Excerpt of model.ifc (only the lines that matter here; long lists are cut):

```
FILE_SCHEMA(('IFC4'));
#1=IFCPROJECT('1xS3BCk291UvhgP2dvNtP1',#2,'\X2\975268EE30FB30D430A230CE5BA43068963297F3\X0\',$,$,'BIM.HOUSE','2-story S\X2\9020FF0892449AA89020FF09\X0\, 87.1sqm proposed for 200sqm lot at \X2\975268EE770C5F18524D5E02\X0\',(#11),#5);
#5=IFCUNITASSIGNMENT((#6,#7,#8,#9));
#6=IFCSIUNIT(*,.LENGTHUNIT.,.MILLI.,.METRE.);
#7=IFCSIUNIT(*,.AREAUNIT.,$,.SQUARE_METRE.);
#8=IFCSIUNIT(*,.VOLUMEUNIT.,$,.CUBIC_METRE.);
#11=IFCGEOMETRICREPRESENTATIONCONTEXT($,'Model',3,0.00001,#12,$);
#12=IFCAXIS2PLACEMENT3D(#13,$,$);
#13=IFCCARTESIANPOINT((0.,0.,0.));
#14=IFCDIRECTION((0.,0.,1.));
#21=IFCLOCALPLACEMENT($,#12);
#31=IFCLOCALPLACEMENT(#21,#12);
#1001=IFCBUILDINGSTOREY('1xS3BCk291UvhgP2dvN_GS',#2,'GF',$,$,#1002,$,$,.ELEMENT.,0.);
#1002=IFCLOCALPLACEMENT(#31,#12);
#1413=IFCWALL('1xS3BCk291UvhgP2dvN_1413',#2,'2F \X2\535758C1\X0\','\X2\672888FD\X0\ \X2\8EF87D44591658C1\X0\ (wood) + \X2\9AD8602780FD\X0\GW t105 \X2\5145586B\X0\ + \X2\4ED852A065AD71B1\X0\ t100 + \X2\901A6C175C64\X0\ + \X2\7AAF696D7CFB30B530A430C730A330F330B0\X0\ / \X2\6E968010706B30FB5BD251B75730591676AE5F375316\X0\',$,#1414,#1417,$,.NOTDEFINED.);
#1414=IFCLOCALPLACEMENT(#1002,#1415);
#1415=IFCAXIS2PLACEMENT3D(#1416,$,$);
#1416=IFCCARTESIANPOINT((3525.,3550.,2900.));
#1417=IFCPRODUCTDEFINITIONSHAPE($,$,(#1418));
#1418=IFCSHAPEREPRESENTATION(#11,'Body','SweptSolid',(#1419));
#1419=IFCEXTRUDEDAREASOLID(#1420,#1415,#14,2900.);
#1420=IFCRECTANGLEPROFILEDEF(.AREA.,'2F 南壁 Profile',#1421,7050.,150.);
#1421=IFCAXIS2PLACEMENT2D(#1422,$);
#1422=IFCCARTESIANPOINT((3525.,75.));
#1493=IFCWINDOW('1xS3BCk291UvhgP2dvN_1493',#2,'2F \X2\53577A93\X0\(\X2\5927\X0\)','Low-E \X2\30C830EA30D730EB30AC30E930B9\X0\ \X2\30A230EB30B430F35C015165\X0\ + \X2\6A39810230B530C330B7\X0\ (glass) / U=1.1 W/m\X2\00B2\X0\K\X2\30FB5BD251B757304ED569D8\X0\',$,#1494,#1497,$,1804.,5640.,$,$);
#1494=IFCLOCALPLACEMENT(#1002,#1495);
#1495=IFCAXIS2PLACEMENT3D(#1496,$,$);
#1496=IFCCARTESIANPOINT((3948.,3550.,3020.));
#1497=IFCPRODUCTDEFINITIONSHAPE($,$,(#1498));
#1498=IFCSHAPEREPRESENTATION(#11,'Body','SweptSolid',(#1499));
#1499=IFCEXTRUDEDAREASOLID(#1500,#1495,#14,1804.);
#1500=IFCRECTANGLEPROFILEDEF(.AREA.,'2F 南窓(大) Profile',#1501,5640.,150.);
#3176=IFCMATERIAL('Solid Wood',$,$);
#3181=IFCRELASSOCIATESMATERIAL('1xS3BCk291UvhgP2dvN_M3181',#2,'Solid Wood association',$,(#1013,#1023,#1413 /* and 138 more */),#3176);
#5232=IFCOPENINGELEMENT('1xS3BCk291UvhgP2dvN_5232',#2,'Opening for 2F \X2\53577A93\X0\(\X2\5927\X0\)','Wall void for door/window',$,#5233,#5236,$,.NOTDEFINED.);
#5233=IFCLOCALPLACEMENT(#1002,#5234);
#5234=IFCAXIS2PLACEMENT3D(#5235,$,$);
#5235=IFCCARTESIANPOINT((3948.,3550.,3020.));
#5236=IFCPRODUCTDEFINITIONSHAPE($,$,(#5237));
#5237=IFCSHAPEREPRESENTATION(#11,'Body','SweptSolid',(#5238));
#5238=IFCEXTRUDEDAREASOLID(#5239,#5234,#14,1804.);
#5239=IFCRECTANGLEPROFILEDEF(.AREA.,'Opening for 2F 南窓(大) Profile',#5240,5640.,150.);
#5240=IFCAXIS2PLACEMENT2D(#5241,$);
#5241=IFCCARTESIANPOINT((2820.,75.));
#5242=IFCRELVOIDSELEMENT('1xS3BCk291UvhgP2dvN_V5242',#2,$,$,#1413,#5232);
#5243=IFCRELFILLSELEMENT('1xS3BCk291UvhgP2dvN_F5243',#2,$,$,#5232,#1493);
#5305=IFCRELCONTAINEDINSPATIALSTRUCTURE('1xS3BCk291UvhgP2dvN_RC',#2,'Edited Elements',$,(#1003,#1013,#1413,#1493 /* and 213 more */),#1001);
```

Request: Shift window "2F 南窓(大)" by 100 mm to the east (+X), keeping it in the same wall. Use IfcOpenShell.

```python
import ifcopenshell
import ifcopenshell.api.geometry
import ifcopenshell.util.placement

model = ifcopenshell.open("model.ifc")

window = model.by_id(1493)
opening = window.FillsVoids[0].RelatingOpeningElement
wall = opening.VoidsElements[0].RelatingBuildingElement

wall_matrix = ifcopenshell.util.placement.get_local_placement(wall.ObjectPlacement)
shift = wall_matrix[:3, 0] * 100.0
before = ifcopenshell.util.placement.get_local_placement(window.ObjectPlacement)[:3, 3].copy()

# The window is not placed relative to its opening, so move both.
for product in (opening, window):
    matrix = ifcopenshell.util.placement.get_local_placement(product.ObjectPlacement)
    matrix[:3, 3] += shift
    ifcopenshell.api.geometry.edit_object_placement(model, product=product, matrix=matrix, is_si=False)

after = ifcopenshell.util.placement.get_local_placement(window.ObjectPlacement)[:3, 3]
print("window moved by", (after - before).round(3) + 0.0)

model.write("model_edited.ifc")
```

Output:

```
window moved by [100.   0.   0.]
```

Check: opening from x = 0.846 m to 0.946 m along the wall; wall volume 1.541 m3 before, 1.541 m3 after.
